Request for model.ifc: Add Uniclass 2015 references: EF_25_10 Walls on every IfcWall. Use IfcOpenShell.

First a look at what the model holds.

```python
import ifcopenshell

model = ifcopenshell.open("model.ifc")
print(model.schema)
print("classifications:", [c.Name for c in model.by_type("IfcClassification")])
for ifc_class in ("IfcDoor", "IfcRoof", "IfcStair", "IfcWall", "IfcWindow"):
    print(ifc_class, len(model.by_type(ifc_class)))
```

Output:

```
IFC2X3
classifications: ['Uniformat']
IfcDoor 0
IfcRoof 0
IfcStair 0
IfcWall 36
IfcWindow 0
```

```python
import ifcopenshell
import ifcopenshell.api.classification

model = ifcopenshell.open("model.ifc")

# IFC2X3 requires Source and Edition and has no link from the project to the system.
system = model.create_entity("IfcClassification", Source="NBS", Edition="2015", Name="Uniclass 2015")

codes = {
    "IfcWall": ("EF_25_10", "Walls"),
}
for ifc_class, (code, name) in codes.items():
    products = model.by_type(ifc_class)
    ifcopenshell.api.classification.add_reference(
        model, products=products, classification=system, identification=code, name=name
    )
    print(code, len(products))

model.write("model_updated.ifc")
```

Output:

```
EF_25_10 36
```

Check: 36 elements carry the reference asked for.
